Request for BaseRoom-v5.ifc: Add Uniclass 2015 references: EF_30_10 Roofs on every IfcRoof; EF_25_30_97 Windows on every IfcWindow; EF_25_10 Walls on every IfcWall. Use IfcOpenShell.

First a look at what the model holds.

```python
import ifcopenshell

model = ifcopenshell.open("BaseRoom-v5.ifc")
print(model.schema)
print("classifications:", [c.Name for c in model.by_type("IfcClassification")])
for ifc_class in ("IfcDoor", "IfcRoof", "IfcStair", "IfcWall", "IfcWindow"):
    print(ifc_class, len(model.by_type(ifc_class)))
```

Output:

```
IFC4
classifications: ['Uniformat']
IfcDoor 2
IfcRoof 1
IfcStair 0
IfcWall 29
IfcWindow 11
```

```python
import ifcopenshell
import ifcopenshell.api.classification

model = ifcopenshell.open("BaseRoom-v5.ifc")

system = ifcopenshell.api.classification.add_classification(model, classification="Uniclass 2015")

codes = {
    "IfcRoof": ("EF_30_10", "Roofs"),
    "IfcWindow": ("EF_25_30_97", "Windows"),
    "IfcWall": ("EF_25_10", "Walls"),
}
for ifc_class, (code, name) in codes.items():
    products = model.by_type(ifc_class)
    ifcopenshell.api.classification.add_reference(
        model, products=products, classification=system, identification=code, name=name
    )
    print(code, len(products))

model.write("BaseRoom-v5_v2.ifc")
```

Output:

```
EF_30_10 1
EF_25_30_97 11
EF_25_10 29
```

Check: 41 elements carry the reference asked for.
